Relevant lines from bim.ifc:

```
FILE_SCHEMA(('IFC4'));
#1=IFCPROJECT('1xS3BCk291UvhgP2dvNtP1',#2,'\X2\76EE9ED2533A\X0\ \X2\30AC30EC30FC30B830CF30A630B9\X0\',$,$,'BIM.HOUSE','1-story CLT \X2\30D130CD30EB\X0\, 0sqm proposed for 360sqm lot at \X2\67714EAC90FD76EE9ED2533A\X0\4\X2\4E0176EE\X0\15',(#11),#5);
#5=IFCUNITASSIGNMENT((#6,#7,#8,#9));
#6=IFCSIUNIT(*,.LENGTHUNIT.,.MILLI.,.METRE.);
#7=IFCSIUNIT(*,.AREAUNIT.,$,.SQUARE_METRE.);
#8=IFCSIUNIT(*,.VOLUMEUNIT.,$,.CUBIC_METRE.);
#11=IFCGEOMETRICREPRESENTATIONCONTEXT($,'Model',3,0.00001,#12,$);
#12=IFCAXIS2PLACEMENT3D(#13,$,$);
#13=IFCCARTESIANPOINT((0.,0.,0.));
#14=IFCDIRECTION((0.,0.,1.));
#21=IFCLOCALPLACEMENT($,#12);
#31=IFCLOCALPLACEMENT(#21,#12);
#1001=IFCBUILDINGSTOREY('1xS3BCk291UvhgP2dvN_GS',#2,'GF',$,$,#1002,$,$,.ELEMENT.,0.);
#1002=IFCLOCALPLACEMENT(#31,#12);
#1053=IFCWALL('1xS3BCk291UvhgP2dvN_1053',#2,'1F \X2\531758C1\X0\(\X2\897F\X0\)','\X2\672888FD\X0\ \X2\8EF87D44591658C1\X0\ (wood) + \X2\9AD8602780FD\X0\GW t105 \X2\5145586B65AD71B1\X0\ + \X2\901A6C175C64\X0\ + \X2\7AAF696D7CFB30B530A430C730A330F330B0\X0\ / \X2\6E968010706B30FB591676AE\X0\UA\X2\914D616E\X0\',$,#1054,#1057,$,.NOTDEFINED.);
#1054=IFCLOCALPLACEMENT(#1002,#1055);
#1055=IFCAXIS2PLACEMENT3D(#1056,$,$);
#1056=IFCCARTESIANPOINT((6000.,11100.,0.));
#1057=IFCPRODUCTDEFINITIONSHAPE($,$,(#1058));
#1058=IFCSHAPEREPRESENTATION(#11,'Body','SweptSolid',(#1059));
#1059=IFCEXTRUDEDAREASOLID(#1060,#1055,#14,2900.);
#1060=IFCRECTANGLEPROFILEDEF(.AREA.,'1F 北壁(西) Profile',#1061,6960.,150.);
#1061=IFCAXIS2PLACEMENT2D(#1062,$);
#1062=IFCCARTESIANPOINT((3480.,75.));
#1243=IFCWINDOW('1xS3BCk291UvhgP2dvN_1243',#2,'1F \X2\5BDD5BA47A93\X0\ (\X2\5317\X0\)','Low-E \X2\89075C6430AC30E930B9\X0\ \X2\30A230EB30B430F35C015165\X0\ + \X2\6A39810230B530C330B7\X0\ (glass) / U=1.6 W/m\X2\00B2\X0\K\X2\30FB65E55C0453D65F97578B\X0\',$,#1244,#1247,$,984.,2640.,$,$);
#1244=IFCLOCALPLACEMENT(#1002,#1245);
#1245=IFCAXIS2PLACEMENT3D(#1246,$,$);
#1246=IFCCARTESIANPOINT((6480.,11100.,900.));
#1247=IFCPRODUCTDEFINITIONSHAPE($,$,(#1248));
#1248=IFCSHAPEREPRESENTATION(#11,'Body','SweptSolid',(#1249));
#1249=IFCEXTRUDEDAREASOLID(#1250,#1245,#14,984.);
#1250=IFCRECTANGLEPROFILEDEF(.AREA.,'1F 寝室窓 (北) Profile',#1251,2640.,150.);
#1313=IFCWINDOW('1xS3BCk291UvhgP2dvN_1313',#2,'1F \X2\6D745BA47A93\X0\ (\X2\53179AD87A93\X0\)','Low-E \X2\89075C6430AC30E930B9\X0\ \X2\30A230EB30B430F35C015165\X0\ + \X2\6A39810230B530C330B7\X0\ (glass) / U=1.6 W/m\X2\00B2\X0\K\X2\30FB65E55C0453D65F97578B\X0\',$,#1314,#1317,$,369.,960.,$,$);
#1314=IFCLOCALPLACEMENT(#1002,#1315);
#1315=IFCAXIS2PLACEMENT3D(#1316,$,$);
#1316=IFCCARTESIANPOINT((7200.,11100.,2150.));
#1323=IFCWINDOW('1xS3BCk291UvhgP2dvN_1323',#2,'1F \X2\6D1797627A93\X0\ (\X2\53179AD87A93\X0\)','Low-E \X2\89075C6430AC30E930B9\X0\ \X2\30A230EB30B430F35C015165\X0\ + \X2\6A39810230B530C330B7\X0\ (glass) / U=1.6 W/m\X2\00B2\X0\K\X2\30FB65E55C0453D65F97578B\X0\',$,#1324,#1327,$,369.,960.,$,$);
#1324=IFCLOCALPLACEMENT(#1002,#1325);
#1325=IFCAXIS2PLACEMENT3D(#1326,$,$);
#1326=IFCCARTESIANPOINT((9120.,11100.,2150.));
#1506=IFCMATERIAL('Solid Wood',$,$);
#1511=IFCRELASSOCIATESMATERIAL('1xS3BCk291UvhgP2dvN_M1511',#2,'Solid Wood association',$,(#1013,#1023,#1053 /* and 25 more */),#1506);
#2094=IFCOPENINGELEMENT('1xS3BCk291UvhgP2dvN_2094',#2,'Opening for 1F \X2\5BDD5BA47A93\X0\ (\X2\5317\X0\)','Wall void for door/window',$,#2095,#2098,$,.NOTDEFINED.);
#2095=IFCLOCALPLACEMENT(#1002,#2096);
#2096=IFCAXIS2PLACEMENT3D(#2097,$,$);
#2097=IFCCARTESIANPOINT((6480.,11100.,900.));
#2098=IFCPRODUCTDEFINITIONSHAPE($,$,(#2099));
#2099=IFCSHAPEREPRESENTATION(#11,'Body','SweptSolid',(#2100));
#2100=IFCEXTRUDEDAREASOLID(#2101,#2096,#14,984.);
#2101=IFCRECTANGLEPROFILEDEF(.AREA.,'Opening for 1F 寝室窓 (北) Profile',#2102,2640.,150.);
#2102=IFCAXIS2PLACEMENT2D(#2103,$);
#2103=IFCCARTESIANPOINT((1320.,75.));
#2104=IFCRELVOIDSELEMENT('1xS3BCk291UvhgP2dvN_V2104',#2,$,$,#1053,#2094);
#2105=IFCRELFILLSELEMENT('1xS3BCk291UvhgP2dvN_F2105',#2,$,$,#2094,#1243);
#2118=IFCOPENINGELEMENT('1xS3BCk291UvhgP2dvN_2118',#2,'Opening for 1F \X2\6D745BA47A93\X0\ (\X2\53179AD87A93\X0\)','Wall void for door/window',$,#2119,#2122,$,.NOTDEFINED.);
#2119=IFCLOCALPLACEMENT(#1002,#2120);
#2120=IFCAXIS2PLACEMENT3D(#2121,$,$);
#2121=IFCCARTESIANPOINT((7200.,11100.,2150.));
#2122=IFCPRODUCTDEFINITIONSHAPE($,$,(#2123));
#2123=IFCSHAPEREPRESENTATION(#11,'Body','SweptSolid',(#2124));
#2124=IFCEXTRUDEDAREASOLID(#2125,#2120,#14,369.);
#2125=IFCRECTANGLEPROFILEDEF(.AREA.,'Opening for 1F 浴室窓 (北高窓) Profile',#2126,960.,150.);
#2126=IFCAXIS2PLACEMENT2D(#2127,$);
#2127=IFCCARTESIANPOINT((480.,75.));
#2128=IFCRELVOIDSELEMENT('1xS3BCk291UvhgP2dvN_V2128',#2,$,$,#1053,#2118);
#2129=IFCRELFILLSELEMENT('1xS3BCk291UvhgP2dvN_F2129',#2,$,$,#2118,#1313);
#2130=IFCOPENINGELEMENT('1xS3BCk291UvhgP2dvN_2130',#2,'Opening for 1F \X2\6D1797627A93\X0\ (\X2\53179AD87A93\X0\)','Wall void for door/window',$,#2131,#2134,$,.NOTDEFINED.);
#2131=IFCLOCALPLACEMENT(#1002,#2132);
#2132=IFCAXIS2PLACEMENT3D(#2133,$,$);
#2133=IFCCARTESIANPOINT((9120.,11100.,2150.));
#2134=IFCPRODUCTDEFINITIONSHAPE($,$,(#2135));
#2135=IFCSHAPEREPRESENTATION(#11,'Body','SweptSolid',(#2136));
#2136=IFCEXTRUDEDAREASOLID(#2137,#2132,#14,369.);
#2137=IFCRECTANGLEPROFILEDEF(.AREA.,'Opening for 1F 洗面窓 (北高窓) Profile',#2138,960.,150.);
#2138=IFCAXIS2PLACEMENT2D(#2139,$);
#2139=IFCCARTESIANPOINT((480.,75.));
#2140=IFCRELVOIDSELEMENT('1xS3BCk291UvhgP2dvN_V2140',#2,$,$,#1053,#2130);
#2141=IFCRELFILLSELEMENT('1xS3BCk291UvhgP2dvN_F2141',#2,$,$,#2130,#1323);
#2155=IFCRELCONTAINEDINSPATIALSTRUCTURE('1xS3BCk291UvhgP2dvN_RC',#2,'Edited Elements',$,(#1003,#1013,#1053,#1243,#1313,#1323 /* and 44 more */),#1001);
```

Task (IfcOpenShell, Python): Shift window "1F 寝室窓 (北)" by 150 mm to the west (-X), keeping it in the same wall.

```python
import ifcopenshell
import ifcopenshell.api.geometry
import ifcopenshell.util.placement
import ifcopenshell.util.unit

model = ifcopenshell.open("bim.ifc")
unit_scale = ifcopenshell.util.unit.calculate_unit_scale(model)

window = model.by_guid("1xS3BCk291UvhgP2dvN_1243")
opening = window.FillsVoids[0].RelatingOpeningElement
wall = opening.VoidsElements[0].RelatingBuildingElement

wall_matrix = ifcopenshell.util.placement.get_local_placement(wall.ObjectPlacement)
shift = wall_matrix[:3, 0] * -0.15 / unit_scale
before = ifcopenshell.util.placement.get_local_placement(window.ObjectPlacement)[:3, 3].copy()

# The window is not placed relative to its opening, so move both.
for product in (opening, window):
    matrix = ifcopenshell.util.placement.get_local_placement(product.ObjectPlacement)
    matrix[:3, 3] += shift
    ifcopenshell.api.geometry.edit_object_placement(model, product=product, matrix=matrix, is_si=False)

after = ifcopenshell.util.placement.get_local_placement(window.ObjectPlacement)[:3, 3]
print("window moved by", (after - before).round(3) + 0.0)

model.write("bim_edited.ifc")
```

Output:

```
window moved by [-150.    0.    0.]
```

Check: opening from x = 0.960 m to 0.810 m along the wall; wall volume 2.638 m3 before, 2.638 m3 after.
